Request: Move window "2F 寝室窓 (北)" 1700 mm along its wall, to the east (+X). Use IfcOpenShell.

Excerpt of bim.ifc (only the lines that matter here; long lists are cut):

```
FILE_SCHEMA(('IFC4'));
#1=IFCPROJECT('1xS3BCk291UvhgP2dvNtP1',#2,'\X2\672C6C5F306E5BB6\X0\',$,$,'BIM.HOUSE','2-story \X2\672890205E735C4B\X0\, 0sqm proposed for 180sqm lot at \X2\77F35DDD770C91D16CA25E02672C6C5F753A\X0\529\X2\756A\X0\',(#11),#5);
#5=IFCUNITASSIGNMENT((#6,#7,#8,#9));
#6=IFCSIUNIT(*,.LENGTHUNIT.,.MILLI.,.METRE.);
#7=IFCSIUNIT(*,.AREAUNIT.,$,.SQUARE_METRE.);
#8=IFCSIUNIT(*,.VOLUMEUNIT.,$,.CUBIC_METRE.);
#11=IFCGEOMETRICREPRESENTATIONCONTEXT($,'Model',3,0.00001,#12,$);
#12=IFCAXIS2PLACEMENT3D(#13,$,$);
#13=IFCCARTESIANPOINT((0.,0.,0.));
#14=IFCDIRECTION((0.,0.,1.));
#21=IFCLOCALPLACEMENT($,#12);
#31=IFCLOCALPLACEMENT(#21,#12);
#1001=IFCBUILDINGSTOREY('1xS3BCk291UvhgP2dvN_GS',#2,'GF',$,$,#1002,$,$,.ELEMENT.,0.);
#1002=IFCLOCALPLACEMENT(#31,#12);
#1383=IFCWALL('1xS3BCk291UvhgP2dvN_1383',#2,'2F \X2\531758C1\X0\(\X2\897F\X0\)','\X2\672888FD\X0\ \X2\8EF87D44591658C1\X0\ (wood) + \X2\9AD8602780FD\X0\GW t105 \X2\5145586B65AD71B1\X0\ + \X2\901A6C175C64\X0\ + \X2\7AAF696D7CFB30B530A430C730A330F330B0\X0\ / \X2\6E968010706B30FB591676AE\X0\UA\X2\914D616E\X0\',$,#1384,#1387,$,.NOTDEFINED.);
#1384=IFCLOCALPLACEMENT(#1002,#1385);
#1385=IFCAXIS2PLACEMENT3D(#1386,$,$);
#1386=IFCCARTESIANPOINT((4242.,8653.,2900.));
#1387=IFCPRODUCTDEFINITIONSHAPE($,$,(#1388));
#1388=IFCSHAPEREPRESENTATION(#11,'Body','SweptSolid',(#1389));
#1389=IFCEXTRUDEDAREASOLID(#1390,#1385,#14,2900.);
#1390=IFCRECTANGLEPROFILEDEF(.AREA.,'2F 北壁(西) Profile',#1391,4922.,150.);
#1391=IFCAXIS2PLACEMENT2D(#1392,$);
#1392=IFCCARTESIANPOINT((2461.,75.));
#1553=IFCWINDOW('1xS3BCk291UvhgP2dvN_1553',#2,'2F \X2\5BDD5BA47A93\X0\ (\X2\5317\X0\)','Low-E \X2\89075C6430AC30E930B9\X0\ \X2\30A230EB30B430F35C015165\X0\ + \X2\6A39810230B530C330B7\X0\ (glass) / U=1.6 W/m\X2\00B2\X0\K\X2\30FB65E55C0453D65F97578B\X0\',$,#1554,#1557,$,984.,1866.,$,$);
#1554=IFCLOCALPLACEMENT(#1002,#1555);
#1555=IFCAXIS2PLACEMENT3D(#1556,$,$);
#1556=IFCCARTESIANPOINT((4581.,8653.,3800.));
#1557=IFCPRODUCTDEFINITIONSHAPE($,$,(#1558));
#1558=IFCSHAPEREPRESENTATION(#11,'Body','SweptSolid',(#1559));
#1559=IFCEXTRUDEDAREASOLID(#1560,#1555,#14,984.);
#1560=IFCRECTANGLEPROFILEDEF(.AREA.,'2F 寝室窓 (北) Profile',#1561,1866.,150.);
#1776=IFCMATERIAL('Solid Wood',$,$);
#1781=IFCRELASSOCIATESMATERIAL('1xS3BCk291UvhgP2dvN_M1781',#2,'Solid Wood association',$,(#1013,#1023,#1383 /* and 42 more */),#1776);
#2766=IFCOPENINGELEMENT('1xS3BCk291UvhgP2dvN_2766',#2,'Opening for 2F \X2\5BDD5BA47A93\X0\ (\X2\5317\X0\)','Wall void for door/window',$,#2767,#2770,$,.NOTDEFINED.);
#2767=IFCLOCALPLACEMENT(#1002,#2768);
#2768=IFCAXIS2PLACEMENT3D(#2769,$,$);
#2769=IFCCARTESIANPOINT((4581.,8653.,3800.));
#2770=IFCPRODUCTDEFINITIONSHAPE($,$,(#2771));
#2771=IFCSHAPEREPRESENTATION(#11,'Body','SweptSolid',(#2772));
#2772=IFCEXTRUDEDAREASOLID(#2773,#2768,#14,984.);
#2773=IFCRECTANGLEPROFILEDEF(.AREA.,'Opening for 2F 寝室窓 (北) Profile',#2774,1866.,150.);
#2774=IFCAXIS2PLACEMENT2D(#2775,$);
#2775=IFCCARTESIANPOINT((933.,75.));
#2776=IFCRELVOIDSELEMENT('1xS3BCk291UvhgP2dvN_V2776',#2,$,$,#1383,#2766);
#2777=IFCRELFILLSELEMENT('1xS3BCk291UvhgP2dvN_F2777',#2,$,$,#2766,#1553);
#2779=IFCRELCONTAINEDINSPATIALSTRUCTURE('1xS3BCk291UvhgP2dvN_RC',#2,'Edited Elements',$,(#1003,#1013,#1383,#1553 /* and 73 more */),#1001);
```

```python
import ifcopenshell
import ifcopenshell.api.geometry
import ifcopenshell.util.placement
import ifcopenshell.util.unit

model = ifcopenshell.open("bim.ifc")
unit_scale = ifcopenshell.util.unit.calculate_unit_scale(model)

window = model.by_guid("1xS3BCk291UvhgP2dvN_1553")
opening = window.FillsVoids[0].RelatingOpeningElement
wall = opening.VoidsElements[0].RelatingBuildingElement

wall_matrix = ifcopenshell.util.placement.get_local_placement(wall.ObjectPlacement)
shift = wall_matrix[:3, 0] * 1.7 / unit_scale
before = ifcopenshell.util.placement.get_local_placement(window.ObjectPlacement)[:3, 3].copy()

# The window is not placed relative to its opening, so move both.
for product in (opening, window):
    matrix = ifcopenshell.util.placement.get_local_placement(product.ObjectPlacement)
    matrix[:3, 3] += shift
    ifcopenshell.api.geometry.edit_object_placement(model, product=product, matrix=matrix, is_si=False)

after = ifcopenshell.util.placement.get_local_placement(window.ObjectPlacement)[:3, 3]
print("window moved by", (after - before).round(3) + 0.0)

model.write("bim-out.ifc")
```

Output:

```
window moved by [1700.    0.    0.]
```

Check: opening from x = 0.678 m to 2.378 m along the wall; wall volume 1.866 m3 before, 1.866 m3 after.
